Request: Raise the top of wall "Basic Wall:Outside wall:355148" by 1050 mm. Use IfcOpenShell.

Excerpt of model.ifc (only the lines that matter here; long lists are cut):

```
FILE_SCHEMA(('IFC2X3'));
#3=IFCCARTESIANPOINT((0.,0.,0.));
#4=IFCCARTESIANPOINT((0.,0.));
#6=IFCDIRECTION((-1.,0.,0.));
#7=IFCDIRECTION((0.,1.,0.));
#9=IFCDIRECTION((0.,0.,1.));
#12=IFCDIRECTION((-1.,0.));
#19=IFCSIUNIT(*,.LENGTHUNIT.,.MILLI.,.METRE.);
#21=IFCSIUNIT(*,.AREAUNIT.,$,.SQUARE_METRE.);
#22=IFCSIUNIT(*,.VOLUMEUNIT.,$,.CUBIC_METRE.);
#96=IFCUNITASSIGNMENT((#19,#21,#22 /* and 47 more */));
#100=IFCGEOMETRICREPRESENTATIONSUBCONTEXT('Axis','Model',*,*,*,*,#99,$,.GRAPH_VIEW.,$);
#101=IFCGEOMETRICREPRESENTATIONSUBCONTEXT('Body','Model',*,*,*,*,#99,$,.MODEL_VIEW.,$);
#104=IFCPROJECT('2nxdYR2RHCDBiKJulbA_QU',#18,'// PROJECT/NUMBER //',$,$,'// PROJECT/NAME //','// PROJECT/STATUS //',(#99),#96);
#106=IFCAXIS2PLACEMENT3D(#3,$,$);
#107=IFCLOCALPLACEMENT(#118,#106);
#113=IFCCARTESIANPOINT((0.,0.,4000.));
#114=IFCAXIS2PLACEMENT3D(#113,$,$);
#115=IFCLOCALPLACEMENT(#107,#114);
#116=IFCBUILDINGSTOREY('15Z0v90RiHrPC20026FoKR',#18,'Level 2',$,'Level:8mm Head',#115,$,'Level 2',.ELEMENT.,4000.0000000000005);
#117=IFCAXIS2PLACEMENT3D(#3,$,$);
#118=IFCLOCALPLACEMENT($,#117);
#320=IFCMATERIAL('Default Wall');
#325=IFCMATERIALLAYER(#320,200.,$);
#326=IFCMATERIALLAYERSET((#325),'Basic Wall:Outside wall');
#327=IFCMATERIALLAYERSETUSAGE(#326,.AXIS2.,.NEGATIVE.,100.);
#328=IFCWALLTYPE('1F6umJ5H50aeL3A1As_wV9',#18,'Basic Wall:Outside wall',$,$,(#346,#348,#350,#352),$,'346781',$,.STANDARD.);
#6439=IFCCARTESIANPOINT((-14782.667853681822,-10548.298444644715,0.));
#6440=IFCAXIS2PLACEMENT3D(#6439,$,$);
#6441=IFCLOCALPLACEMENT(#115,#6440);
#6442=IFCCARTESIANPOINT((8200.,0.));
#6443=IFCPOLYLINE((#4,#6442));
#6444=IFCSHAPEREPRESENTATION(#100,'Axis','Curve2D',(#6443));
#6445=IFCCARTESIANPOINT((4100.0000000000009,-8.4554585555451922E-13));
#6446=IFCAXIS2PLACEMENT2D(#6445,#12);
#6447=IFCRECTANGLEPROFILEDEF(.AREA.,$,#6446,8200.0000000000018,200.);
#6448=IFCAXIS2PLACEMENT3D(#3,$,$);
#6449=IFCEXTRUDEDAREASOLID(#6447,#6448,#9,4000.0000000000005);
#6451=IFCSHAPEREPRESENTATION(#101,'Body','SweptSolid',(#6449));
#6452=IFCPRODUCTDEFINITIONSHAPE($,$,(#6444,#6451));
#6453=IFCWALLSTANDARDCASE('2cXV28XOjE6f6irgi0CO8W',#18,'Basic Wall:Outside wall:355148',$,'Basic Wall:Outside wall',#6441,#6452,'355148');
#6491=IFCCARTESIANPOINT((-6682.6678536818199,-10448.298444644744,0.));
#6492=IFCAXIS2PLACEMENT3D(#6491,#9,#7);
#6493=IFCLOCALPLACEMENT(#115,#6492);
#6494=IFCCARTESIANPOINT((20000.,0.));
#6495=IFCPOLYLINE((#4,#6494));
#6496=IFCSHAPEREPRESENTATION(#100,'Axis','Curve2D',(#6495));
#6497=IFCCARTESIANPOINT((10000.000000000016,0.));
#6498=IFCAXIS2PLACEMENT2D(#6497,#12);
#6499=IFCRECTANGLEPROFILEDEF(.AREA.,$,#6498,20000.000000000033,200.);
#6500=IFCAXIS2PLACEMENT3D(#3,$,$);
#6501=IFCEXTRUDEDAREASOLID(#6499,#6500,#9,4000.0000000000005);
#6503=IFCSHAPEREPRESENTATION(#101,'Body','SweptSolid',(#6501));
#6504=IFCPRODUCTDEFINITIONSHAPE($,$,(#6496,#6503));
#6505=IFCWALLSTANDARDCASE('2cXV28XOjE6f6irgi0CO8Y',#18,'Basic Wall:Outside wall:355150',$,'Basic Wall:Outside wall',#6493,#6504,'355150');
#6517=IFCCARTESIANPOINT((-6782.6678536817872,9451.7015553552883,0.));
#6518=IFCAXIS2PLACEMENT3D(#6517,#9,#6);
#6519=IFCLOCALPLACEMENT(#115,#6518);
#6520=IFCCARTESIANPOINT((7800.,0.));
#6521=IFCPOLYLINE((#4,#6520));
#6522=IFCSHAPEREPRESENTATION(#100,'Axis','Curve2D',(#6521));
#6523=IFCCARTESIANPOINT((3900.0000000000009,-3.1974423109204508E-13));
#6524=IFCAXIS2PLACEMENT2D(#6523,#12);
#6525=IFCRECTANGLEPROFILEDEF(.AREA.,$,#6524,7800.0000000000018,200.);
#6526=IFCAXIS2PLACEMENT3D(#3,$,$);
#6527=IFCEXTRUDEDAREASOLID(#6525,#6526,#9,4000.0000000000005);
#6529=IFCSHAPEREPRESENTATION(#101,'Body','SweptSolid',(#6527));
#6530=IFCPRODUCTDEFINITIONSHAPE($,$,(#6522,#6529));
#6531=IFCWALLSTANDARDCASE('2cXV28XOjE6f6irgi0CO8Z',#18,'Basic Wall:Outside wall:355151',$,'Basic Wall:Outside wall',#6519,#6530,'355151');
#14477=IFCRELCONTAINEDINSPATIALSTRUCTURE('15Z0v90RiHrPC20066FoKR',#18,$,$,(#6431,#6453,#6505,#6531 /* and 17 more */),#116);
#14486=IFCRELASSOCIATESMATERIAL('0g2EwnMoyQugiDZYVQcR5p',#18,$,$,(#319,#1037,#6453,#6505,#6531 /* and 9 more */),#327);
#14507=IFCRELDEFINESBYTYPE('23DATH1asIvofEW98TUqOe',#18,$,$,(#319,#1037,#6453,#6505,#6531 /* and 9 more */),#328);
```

```python
import ifcopenshell
import ifcopenshell.geom
import ifcopenshell.util.representation
import ifcopenshell.util.shape

model = ifcopenshell.open("model.ifc")
settings = ifcopenshell.geom.settings()


def volume(element):
    """Net volume in cubic metres, openings subtracted."""
    shape = ifcopenshell.geom.create_shape(settings, element)
    return ifcopenshell.util.shape.get_volume(shape.geometry)


wall = model.by_guid("2cXV28XOjE6f6irgi0CO8W")
before = volume(wall)

body = ifcopenshell.util.representation.get_representation(wall, "Model", "Body")
solid = body.Items[0]
old_height = solid.Depth
solid.Depth += 1050.0
after = volume(wall)

print(f"height {old_height:g} -> {solid.Depth:g}, volume {before:.3f} -> {after:.3f} m3")

model.write("model_v2.ifc")
```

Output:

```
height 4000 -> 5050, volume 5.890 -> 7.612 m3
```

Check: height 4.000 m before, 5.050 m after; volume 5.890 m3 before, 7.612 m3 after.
